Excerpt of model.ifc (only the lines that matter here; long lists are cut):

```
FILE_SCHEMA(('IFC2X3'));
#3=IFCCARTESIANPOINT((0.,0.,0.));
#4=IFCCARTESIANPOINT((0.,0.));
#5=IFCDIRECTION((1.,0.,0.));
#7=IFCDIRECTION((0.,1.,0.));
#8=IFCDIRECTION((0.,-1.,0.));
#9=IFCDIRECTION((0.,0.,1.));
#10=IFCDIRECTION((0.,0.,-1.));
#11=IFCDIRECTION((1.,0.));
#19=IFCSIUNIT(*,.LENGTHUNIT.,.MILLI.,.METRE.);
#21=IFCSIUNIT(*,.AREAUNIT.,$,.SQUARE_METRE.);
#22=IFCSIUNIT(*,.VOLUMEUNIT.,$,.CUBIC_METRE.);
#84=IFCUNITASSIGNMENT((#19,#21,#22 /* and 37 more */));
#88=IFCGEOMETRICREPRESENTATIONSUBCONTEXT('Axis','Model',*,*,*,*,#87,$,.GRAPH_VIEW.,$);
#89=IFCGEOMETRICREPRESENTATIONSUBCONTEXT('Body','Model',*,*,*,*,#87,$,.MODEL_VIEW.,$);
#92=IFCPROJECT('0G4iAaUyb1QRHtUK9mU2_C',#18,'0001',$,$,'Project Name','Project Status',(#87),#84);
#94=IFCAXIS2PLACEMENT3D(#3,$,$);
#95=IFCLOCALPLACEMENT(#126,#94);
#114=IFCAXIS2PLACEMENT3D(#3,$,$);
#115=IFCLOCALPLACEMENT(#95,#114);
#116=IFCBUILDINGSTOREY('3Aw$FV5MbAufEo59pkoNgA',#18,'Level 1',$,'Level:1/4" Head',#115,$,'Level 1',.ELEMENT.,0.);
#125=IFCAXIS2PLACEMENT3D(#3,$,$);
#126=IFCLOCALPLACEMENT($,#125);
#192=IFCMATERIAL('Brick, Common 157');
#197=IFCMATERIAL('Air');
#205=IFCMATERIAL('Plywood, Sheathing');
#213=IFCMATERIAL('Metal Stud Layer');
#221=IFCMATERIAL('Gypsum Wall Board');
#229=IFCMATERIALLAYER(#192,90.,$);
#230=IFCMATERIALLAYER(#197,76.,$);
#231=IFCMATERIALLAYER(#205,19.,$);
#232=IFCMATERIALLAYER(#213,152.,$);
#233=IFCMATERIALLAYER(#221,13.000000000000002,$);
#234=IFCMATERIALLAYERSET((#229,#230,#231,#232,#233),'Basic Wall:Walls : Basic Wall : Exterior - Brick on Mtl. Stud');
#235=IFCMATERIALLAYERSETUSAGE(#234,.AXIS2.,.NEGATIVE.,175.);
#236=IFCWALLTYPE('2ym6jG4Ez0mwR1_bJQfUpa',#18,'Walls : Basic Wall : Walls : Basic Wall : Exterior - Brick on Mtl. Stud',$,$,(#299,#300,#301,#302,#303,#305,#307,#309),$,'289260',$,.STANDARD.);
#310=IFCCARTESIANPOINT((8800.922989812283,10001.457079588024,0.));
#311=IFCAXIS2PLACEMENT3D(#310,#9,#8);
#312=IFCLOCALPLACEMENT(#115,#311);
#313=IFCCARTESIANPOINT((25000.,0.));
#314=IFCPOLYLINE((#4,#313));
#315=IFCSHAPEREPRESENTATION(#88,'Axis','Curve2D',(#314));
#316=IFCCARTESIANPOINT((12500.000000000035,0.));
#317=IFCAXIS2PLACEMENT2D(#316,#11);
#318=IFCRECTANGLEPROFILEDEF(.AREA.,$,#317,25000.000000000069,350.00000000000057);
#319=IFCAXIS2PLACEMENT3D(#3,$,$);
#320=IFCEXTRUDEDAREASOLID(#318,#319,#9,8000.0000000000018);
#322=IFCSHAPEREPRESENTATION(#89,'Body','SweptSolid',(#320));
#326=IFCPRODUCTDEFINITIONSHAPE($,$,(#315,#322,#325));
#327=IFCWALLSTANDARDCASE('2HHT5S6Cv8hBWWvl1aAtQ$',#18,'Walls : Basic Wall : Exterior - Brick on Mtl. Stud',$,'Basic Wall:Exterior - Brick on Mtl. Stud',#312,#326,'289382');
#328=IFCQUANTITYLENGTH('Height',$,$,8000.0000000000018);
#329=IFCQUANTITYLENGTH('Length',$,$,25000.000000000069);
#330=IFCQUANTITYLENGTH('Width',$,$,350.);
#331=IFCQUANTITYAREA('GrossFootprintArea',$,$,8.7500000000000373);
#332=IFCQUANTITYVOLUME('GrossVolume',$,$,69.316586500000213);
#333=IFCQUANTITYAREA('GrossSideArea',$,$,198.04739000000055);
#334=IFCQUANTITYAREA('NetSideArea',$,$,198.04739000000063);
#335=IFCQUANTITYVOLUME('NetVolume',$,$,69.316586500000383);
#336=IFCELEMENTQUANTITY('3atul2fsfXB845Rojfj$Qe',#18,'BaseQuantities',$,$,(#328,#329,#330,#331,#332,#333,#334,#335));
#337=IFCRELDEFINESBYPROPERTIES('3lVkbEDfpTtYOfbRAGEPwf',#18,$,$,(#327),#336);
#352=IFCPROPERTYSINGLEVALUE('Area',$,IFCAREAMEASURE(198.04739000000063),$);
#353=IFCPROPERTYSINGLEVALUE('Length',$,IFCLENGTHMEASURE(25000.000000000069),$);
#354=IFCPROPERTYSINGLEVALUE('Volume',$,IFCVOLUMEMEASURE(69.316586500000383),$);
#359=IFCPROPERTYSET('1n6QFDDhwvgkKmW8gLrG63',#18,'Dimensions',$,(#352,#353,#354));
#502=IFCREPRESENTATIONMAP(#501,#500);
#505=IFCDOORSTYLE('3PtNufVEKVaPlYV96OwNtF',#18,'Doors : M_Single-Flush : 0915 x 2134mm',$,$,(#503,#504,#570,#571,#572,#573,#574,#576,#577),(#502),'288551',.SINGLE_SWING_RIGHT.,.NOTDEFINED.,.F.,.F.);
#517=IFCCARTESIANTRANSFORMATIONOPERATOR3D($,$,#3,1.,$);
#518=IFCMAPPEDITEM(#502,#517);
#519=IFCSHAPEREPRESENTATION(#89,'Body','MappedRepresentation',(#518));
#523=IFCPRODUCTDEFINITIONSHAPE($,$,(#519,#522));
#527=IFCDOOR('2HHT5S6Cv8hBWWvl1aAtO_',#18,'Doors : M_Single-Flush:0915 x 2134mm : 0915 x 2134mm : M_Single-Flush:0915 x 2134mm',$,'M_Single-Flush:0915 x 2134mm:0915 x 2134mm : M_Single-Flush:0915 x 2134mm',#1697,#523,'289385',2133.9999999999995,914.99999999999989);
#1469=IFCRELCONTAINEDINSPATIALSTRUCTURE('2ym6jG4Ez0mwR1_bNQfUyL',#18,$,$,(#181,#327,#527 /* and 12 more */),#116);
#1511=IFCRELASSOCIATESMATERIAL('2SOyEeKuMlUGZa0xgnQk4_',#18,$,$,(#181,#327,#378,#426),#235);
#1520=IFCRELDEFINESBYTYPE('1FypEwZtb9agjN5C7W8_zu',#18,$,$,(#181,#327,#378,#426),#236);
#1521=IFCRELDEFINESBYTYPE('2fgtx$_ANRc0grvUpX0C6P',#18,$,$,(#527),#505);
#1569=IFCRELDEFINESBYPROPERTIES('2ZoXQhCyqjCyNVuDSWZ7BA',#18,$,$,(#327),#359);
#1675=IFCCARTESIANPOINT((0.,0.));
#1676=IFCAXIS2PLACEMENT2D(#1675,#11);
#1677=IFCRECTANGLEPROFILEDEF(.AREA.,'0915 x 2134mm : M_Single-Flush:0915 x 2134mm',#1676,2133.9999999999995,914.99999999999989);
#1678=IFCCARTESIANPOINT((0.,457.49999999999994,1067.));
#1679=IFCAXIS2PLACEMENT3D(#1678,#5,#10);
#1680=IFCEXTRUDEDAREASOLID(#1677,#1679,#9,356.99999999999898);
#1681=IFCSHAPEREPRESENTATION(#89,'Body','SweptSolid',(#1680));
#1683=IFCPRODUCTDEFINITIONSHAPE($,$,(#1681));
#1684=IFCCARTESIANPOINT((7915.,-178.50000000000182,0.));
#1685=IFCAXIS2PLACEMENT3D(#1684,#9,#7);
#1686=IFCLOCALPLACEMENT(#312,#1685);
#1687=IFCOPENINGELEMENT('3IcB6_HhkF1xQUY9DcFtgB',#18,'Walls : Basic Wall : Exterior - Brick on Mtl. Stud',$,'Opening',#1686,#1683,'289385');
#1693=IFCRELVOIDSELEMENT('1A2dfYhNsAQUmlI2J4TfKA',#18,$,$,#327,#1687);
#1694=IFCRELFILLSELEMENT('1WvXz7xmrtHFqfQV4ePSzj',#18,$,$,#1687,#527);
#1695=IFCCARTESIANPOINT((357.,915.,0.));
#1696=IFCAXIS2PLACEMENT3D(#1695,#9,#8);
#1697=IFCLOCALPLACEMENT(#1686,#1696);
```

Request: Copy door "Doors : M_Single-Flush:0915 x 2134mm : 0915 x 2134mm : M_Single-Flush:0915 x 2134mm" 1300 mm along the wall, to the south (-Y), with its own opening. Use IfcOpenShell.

```python
import ifcopenshell
import ifcopenshell.api.feature
import ifcopenshell.api.geometry
import ifcopenshell.api.pset
import ifcopenshell.api.root
import ifcopenshell.geom
import ifcopenshell.util.element
import ifcopenshell.util.placement
import ifcopenshell.util.shape
import ifcopenshell.util.unit

model = ifcopenshell.open("model.ifc")
unit_scale = ifcopenshell.util.unit.calculate_unit_scale(model)
area_scale = ifcopenshell.util.unit.calculate_unit_scale(model, "AREAUNIT")
volume_scale = ifcopenshell.util.unit.calculate_unit_scale(model, "VOLUMEUNIT")
settings = ifcopenshell.geom.settings()


def volume(element):
    """Net volume in cubic metres, openings subtracted."""
    shape = ifcopenshell.geom.create_shape(settings, element)
    return ifcopenshell.util.shape.get_volume(shape.geometry)


def reuse_history(source, copy):
    """copy_class also copies each property set's owner history, people and application; keep the originals."""
    for rel in copy.IsDefinedBy:
        if rel.is_a("IfcRelDefinesByProperties") and (history := rel.RelatingPropertyDefinition.OwnerHistory):
            rel.RelatingPropertyDefinition.OwnerHistory = source.OwnerHistory
            ifcopenshell.util.element.remove_deep2(model, history)


door = model.by_id(527)
opening = door.FillsVoids[0].RelatingOpeningElement
wall = opening.VoidsElements[0].RelatingBuildingElement
before = volume(wall)
shift = ifcopenshell.util.placement.get_local_placement(wall.ObjectPlacement)[:3, 0] * 1.3 / unit_scale

# copy_class copies the void relationship, type, container and properties, but no geometry.
new_opening = ifcopenshell.api.root.copy_class(model, product=opening)
new_opening.Representation = ifcopenshell.util.element.copy_deep(
    model, opening.Representation, exclude=["IfcGeometricRepresentationContext", "IfcRepresentationMap"]
)
new_opening.Tag = None
reuse_history(opening, new_opening)
new_door = ifcopenshell.api.root.copy_class(model, product=door)
new_door.Representation = ifcopenshell.util.element.copy_deep(
    model, door.Representation, exclude=["IfcGeometricRepresentationContext", "IfcRepresentationMap"]
)
new_door.Tag = None
reuse_history(door, new_door)
fills = ifcopenshell.api.feature.add_filling(model, opening=new_opening, element=new_door)
fills.OwnerHistory = new_door.OwnerHistory  # required in IFC2X3

for old, new in ((opening, new_opening), (door, new_door)):
    matrix = ifcopenshell.util.placement.get_local_placement(old.ObjectPlacement)
    matrix[:3, 3] += shift
    ifcopenshell.api.geometry.edit_object_placement(model, product=new, matrix=matrix, is_si=False)

after = volume(wall)
thickness = 0.35  # wall thickness in metres

# Update the wall's stored quantities.
qto = model.by_id(ifcopenshell.util.element.get_pset(wall, "BaseQuantities", should_inherit=False)["id"])
ifcopenshell.api.pset.edit_qto(model, qto=qto, properties={
    "NetSideArea": after / thickness / area_scale,
    "NetVolume": after / volume_scale,
})
pset = model.by_id(ifcopenshell.util.element.get_pset(wall, "Dimensions", should_inherit=False)["id"])
ifcopenshell.api.pset.edit_pset(model, pset=pset, properties={
    "Area": model.create_entity("IfcAreaMeasure", after / thickness / area_scale),
    "Volume": model.create_entity("IfcVolumeMeasure", after / volume_scale),
})

print(f"wall volume {before:.3f} -> {after:.3f} m3")

model.write("model_edited.ifc")
```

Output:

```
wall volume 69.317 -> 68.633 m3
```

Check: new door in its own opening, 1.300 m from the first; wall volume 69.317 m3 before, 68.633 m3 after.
